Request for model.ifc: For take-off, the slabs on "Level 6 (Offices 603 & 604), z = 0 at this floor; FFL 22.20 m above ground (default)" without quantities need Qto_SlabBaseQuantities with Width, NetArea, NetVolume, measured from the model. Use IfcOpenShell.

First a look at what the model holds.

```python
import ifcopenshell
import ifcopenshell.util.element
import ifcopenshell.util.unit

model = ifcopenshell.open("model.ifc")
print(model.schema)
for unit_type in ("LENGTHUNIT", "AREAUNIT", "VOLUMEUNIT"):
    print(unit_type, ifcopenshell.util.unit.calculate_unit_scale(model, unit_type))
storey = next(s for s in model.by_type("IfcBuildingStorey") if s.Name == "Level 6 (Offices 603 & 604), z = 0 at this floor; FFL 22.20 m above ground (default)")
slabs = [e for e in ifcopenshell.util.element.get_decomposition(storey) if e.is_a("IfcSlab")]
for e in sorted(slabs, key=lambda e: e.id()):
    print(e.id(), e.is_a(), e.Name, list(ifcopenshell.util.element.get_psets(e, qtos_only=True)), sep=" | ")
```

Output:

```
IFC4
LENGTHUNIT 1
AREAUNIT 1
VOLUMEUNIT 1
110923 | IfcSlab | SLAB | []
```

```python
import ifcopenshell
import ifcopenshell.api.pset
import ifcopenshell.geom
import ifcopenshell.util.element
import ifcopenshell.util.shape
import ifcopenshell.util.unit

model = ifcopenshell.open("model.ifc")
unit_scale = ifcopenshell.util.unit.calculate_unit_scale(model)
area_scale = ifcopenshell.util.unit.calculate_unit_scale(model, "AREAUNIT")
volume_scale = ifcopenshell.util.unit.calculate_unit_scale(model, "VOLUMEUNIT")
settings = ifcopenshell.geom.settings()

storey = next(s for s in model.by_type("IfcBuildingStorey") if s.Name == "Level 6 (Offices 603 & 604), z = 0 at this floor; FFL 22.20 m above ground (default)")
slabs = [e for e in ifcopenshell.util.element.get_decomposition(storey) if e.is_a("IfcSlab")]

for e in sorted(slabs, key=lambda e: e.id()):
    if ifcopenshell.util.element.get_psets(e, qtos_only=True, should_inherit=False):
        continue
    # Geometry comes back in metres, in the element's own axes.
    shape = ifcopenshell.geom.create_shape(settings, e)
    values = {
        "Width": ifcopenshell.util.shape.get_z(shape.geometry) / unit_scale,
        "NetArea": ifcopenshell.util.shape.get_footprint_area(shape.geometry) / area_scale,
        "NetVolume": ifcopenshell.util.shape.get_volume(shape.geometry) / volume_scale,
    }
    qto = ifcopenshell.api.pset.add_qto(model, product=e, name="Qto_SlabBaseQuantities")
    ifcopenshell.api.pset.edit_qto(model, qto=qto, properties=values)
    print(e.id(), {k: round(v, 3) for k, v in values.items()})

model.write("model_edited.ifc")
```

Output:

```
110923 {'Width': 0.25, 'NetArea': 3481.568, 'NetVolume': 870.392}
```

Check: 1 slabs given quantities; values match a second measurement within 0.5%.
